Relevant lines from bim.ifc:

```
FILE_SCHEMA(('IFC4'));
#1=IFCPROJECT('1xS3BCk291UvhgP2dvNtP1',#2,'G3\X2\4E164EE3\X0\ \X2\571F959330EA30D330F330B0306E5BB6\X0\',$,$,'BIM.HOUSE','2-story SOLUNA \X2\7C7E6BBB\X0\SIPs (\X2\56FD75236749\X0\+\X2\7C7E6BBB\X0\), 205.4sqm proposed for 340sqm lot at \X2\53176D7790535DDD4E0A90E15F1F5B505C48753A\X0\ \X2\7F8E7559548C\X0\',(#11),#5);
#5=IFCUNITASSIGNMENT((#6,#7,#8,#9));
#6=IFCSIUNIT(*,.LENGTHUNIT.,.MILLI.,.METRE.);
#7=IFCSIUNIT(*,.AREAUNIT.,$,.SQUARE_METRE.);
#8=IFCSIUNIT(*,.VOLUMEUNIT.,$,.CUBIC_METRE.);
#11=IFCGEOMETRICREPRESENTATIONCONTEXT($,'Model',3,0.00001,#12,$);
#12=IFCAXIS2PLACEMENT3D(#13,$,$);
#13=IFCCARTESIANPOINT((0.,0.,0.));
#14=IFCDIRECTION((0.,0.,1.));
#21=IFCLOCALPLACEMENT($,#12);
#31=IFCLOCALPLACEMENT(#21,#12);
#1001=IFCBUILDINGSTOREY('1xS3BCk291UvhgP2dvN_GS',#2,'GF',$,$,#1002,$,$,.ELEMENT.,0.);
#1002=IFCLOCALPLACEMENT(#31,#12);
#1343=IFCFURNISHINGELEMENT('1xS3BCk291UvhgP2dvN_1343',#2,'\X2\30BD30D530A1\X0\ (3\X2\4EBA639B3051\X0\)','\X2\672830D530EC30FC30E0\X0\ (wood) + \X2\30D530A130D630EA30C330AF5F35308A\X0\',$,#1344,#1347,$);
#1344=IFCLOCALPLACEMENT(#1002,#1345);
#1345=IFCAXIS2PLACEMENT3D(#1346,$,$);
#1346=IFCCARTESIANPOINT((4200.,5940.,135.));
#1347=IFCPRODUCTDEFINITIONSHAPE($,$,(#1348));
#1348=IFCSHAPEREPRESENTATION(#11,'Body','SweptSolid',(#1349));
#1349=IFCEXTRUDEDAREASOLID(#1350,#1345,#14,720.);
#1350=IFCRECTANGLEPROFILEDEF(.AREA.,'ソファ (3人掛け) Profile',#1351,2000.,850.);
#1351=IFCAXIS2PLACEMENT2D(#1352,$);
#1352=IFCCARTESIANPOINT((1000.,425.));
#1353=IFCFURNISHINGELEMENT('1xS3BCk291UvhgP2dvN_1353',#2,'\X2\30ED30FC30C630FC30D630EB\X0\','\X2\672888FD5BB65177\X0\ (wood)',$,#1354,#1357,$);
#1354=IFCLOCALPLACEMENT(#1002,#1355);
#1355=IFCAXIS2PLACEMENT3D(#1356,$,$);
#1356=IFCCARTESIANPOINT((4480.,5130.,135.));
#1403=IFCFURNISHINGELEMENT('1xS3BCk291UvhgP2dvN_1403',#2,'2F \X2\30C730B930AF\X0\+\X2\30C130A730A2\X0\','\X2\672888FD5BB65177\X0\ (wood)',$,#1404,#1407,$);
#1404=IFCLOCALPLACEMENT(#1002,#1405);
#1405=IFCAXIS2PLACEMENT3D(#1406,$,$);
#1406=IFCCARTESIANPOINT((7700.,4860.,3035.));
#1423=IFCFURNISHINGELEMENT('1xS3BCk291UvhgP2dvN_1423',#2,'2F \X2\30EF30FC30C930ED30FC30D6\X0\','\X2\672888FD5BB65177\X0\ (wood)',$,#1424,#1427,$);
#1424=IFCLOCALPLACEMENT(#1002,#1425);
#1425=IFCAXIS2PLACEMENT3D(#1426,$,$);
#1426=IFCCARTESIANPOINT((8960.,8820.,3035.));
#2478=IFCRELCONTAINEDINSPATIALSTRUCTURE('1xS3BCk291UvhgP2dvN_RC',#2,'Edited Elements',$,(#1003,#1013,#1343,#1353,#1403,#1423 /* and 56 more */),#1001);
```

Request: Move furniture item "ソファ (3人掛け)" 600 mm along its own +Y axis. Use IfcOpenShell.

```python
import ifcopenshell
import ifcopenshell.api.geometry
import ifcopenshell.util.placement
import ifcopenshell.util.unit

model = ifcopenshell.open("bim.ifc")
unit_scale = ifcopenshell.util.unit.calculate_unit_scale(model)

item = model.by_id(1343)
matrix = ifcopenshell.util.placement.get_local_placement(item.ObjectPlacement)
matrix[:3, 3] += matrix[:3, 1] * 0.6 / unit_scale
ifcopenshell.api.geometry.edit_object_placement(model, product=item, matrix=matrix, is_si=False)

print(ifcopenshell.util.placement.get_local_placement(item.ObjectPlacement).round(3) + 0.0)

model.write("bim_v2.ifc")
```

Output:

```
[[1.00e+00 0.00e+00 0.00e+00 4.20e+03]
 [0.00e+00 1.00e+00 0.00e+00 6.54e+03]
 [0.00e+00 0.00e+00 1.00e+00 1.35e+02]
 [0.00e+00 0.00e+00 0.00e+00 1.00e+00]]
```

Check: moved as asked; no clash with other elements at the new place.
